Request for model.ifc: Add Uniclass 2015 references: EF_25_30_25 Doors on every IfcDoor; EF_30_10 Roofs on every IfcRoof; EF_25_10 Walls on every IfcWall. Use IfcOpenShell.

First a look at what the model holds.

```python
import ifcopenshell

model = ifcopenshell.open("model.ifc")
print(model.schema)
print("classifications:", [c.Name for c in model.by_type("IfcClassification")])
for ifc_class in ("IfcDoor", "IfcRoof", "IfcStair", "IfcWall", "IfcWindow"):
    print(ifc_class, len(model.by_type(ifc_class)))
```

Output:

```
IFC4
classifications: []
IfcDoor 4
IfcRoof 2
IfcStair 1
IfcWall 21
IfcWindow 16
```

```python
import ifcopenshell
import ifcopenshell.api.classification

model = ifcopenshell.open("model.ifc")

system = ifcopenshell.api.classification.add_classification(model, classification="Uniclass 2015")

codes = {
    "IfcDoor": ("EF_25_30_25", "Doors"),
    "IfcRoof": ("EF_30_10", "Roofs"),
    "IfcWall": ("EF_25_10", "Walls"),
}
for ifc_class, (code, name) in codes.items():
    products = model.by_type(ifc_class)
    ifcopenshell.api.classification.add_reference(
        model, products=products, classification=system, identification=code, name=name
    )
    print(code, len(products))

model.write("model-out.ifc")
```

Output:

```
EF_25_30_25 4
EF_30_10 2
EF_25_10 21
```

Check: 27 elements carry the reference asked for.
